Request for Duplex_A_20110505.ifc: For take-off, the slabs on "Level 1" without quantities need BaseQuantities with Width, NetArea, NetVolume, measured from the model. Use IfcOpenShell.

First a look at what the model holds.

```python
import ifcopenshell
import ifcopenshell.util.element
import ifcopenshell.util.unit

model = ifcopenshell.open("Duplex_A_20110505.ifc")
print(model.schema)
for unit_type in ("LENGTHUNIT", "AREAUNIT", "VOLUMEUNIT"):
    print(unit_type, ifcopenshell.util.unit.calculate_unit_scale(model, unit_type))
storey = next(s for s in model.by_type("IfcBuildingStorey") if s.Name == "Level 1")
slabs = [e for e in ifcopenshell.util.element.get_decomposition(storey) if e.is_a("IfcSlab")]
for e in sorted(slabs, key=lambda e: e.id()):
    print(e.id(), e.is_a(), e.Name, list(ifcopenshell.util.element.get_psets(e, qtos_only=True)), sep=" | ")
```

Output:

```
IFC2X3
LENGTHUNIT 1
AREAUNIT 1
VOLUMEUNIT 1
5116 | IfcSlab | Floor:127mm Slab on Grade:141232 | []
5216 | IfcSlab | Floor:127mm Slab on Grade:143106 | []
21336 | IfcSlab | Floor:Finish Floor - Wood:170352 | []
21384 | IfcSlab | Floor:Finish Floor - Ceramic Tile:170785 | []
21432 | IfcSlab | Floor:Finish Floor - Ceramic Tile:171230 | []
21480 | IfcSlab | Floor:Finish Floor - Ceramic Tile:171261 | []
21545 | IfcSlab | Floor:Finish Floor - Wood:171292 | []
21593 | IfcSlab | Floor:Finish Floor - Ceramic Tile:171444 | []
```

```python
import ifcopenshell
import ifcopenshell.api.pset
import ifcopenshell.geom
import ifcopenshell.util.element
import ifcopenshell.util.shape
import ifcopenshell.util.unit

model = ifcopenshell.open("Duplex_A_20110505.ifc")
unit_scale = ifcopenshell.util.unit.calculate_unit_scale(model)
area_scale = ifcopenshell.util.unit.calculate_unit_scale(model, "AREAUNIT")
volume_scale = ifcopenshell.util.unit.calculate_unit_scale(model, "VOLUMEUNIT")
settings = ifcopenshell.geom.settings()

storey = next(s for s in model.by_type("IfcBuildingStorey") if s.Name == "Level 1")
slabs = [e for e in ifcopenshell.util.element.get_decomposition(storey) if e.is_a("IfcSlab")]

for e in sorted(slabs, key=lambda e: e.id()):
    if ifcopenshell.util.element.get_psets(e, qtos_only=True, should_inherit=False):
        continue
    # Geometry comes back in metres, in the element's own axes.
    shape = ifcopenshell.geom.create_shape(settings, e)
    values = {
        "Width": ifcopenshell.util.shape.get_z(shape.geometry) / unit_scale,
        "NetArea": ifcopenshell.util.shape.get_footprint_area(shape.geometry) / area_scale,
        "NetVolume": ifcopenshell.util.shape.get_volume(shape.geometry) / volume_scale,
    }
    qto = ifcopenshell.api.pset.add_qto(model, product=e, name="BaseQuantities")
    ifcopenshell.api.pset.edit_qto(model, qto=qto, properties=values)
    print(e.id(), {k: round(v, 3) for k, v in values.items()})

model.write("Duplex_A_20110505_edited.ifc")
```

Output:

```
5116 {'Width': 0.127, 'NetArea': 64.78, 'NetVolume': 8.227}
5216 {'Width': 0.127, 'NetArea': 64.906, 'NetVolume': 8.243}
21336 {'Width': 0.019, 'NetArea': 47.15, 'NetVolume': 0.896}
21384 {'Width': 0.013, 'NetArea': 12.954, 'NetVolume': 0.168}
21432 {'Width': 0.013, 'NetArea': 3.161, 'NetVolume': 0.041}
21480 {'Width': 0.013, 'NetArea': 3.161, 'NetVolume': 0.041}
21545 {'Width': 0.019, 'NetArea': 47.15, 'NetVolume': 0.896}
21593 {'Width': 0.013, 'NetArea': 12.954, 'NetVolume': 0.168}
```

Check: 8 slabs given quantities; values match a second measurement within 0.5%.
